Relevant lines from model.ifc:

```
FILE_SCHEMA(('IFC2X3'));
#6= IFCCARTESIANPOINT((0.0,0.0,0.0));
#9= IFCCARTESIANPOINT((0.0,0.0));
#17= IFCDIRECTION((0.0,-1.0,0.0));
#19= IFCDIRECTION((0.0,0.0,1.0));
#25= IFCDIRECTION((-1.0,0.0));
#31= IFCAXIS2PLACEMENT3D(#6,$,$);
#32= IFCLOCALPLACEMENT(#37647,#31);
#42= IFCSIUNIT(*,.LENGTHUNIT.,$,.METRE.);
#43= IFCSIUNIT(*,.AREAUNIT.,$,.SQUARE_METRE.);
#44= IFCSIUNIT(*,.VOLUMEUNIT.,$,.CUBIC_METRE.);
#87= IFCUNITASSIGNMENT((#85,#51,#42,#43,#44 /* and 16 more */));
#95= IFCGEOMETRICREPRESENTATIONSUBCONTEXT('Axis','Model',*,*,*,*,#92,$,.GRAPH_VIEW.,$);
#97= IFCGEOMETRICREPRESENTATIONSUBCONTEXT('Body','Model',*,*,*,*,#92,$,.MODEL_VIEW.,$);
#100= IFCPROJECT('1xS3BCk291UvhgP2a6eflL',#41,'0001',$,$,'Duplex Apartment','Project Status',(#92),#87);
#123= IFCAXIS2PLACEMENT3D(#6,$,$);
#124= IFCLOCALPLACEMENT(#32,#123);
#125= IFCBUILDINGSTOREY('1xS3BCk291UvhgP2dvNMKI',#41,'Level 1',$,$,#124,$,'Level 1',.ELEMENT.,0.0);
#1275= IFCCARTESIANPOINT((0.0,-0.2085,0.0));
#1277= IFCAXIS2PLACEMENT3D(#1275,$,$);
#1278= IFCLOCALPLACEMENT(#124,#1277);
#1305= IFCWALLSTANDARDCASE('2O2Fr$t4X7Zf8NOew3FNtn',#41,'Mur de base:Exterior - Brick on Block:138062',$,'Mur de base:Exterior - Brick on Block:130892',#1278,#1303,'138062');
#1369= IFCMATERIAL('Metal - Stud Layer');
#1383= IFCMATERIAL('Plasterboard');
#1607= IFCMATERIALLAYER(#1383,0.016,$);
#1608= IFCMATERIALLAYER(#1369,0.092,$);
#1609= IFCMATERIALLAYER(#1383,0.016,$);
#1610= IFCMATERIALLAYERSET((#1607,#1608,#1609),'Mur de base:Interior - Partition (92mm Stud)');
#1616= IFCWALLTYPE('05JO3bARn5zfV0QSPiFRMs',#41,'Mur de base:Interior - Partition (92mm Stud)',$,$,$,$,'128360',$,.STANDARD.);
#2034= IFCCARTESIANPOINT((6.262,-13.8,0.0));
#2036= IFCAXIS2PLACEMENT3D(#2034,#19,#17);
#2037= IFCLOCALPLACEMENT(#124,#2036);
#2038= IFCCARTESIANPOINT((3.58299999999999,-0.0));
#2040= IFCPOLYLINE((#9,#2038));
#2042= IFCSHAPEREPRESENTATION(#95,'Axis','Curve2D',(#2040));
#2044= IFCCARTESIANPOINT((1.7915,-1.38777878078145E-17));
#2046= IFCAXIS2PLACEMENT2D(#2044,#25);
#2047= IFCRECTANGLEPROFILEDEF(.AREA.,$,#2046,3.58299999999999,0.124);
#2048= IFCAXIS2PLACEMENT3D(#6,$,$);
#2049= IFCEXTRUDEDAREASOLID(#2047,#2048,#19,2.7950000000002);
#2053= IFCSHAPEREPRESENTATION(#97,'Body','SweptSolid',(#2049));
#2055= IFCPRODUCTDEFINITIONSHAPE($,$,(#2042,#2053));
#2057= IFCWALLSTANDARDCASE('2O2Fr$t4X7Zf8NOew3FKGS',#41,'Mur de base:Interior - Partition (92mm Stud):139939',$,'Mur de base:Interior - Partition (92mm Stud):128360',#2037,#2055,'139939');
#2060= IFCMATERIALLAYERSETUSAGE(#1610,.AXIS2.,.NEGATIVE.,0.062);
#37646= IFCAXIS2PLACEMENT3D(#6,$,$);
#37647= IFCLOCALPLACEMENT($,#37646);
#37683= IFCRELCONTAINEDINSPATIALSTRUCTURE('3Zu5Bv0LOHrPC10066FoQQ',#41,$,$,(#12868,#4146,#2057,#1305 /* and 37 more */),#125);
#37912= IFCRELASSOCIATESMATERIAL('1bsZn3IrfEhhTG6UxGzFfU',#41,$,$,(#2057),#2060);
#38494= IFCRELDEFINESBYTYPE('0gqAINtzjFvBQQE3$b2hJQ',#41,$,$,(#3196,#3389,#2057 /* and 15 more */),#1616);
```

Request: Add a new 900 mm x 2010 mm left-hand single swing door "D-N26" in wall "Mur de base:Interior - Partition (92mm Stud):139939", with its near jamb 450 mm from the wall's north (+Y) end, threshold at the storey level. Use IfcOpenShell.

```python
import numpy as np
import ifcopenshell
import ifcopenshell.api.feature
import ifcopenshell.api.geometry
import ifcopenshell.api.root
import ifcopenshell.api.spatial
import ifcopenshell.api.type
import ifcopenshell.geom
import ifcopenshell.util.element
import ifcopenshell.util.placement
import ifcopenshell.util.representation
import ifcopenshell.util.shape
import ifcopenshell.util.unit

model = ifcopenshell.open("model.ifc")
unit_scale = ifcopenshell.util.unit.calculate_unit_scale(model)
settings = ifcopenshell.geom.settings()


def volume(element):
    """Net volume in cubic metres, openings subtracted."""
    shape = ifcopenshell.geom.create_shape(settings, element)
    return ifcopenshell.util.shape.get_volume(shape.geometry)


wall = model.by_id(2057)
storey = ifcopenshell.util.element.get_container(wall, ifc_class="IfcBuildingStorey")
context = ifcopenshell.util.representation.get_context(model, "Model", "Body", "MODEL_VIEW")
before = volume(wall)

width, height, from_end, sill = 0.9, 2.01, 0.45, 0.0  # metres

# The wall runs along its own X axis, and the end named is its -X end.
wall_shape = ifcopenshell.geom.create_shape(settings, wall)
x, y, z = ifcopenshell.util.shape.get_vertices(wall_shape.geometry).T
start = x.min() + from_end
face, thickness = float(y.min()), float(y.max() - y.min())
wall_matrix = ifcopenshell.util.placement.get_local_placement(wall.ObjectPlacement)
level = ifcopenshell.util.placement.get_local_placement(storey.ObjectPlacement)[2, 3]


def in_wall(x, y):
    """Placement at x, y metres in the wall's axes, at sill height."""
    matrix = wall_matrix.copy()
    matrix[:, 3] = wall_matrix @ np.array([x / unit_scale, y / unit_scale, 0.0, 1.0])
    matrix[2, 3] = level + sill / unit_scale
    return matrix


# Opening: a box that overshoots both wall faces by 50 mm.
opening = ifcopenshell.api.root.create_entity(model, ifc_class="IfcOpeningElement")
box = ifcopenshell.api.geometry.add_wall_representation(
    model, context=context, length=width, height=height, thickness=thickness + 0.1
)
ifcopenshell.api.geometry.assign_representation(model, product=opening, representation=box)
ifcopenshell.api.geometry.edit_object_placement(model, product=opening, matrix=in_wall(start, face - 0.05), is_si=False)
ifcopenshell.api.feature.add_feature(model, feature=opening, element=wall)

door = ifcopenshell.api.root.create_entity(model, ifc_class="IfcDoor", name="D-N26")
door.OverallWidth, door.OverallHeight = width / unit_scale, height / unit_scale
body = ifcopenshell.api.geometry.add_door_representation(
    model,
    context=context,
    overall_width=door.OverallWidth,
    overall_height=door.OverallHeight,
    operation_type="SINGLE_SWING_LEFT",
    lining_properties={"LiningDepth": thickness / unit_scale, "ThresholdDepth": thickness / unit_scale},
)
ifcopenshell.api.geometry.assign_representation(model, product=door, representation=body)
ifcopenshell.api.spatial.assign_container(model, products=[door], relating_structure=storey)
fills = ifcopenshell.api.feature.add_filling(model, opening=opening, element=door)
fills.OwnerHistory = door.OwnerHistory  # required in IFC2X3

# IFC2X3 keeps the operation on the door style.
style = ifcopenshell.api.root.create_entity(model, ifc_class="IfcDoorStyle", name="D-N26")
style.OperationType, style.ConstructionType = "SINGLE_SWING_LEFT", "NOTDEFINED"
style.ParameterTakesPrecedence = style.Sizeable = False
ifcopenshell.api.type.assign_type(model, related_objects=[door], relating_type=style)

# The lining spans the wall, so the door starts at the wall face.
ifcopenshell.api.geometry.edit_object_placement(model, product=door, matrix=in_wall(start, face), is_si=False)

after = volume(wall)

print(f"wall volume {before:.3f} -> {after:.3f} m3")

model.write("model_v2.ifc")
```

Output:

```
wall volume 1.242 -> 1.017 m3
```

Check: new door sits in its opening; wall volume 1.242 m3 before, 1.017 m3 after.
